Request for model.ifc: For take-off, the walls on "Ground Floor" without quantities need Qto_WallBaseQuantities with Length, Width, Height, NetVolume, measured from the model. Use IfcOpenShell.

First a look at what the model holds.

```python
import ifcopenshell
import ifcopenshell.util.element
import ifcopenshell.util.unit

model = ifcopenshell.open("model.ifc")
print(model.schema)
for unit_type in ("LENGTHUNIT", "AREAUNIT", "VOLUMEUNIT"):
    print(unit_type, ifcopenshell.util.unit.calculate_unit_scale(model, unit_type))
storey = next(s for s in model.by_type("IfcBuildingStorey") if s.Name == "Ground Floor")
walls = [e for e in ifcopenshell.util.element.get_decomposition(storey) if e.is_a("IfcWall")]
for e in sorted(walls, key=lambda e: e.id()):
    print(e.id(), e.is_a(), e.Name, list(ifcopenshell.util.element.get_psets(e, qtos_only=True)), sep=" | ")
```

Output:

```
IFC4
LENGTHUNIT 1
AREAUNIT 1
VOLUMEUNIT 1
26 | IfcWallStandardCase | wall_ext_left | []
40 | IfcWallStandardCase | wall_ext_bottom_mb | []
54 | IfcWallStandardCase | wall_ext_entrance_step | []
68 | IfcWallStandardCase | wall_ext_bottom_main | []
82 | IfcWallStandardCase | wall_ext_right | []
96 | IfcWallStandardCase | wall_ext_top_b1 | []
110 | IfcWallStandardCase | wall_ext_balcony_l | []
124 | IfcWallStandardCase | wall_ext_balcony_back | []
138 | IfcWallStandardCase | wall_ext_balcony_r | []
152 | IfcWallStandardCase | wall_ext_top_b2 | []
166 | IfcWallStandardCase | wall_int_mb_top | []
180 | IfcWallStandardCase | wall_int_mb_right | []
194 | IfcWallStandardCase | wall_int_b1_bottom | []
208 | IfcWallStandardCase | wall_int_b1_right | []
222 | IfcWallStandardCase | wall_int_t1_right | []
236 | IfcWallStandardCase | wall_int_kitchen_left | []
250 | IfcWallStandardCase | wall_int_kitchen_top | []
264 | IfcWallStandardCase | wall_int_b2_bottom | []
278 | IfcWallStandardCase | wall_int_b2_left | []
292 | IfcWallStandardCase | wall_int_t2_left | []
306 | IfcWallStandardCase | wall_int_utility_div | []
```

```python
import ifcopenshell
import ifcopenshell.api.pset
import ifcopenshell.geom
import ifcopenshell.util.element
import ifcopenshell.util.shape
import ifcopenshell.util.unit

model = ifcopenshell.open("model.ifc")
unit_scale = ifcopenshell.util.unit.calculate_unit_scale(model)
volume_scale = ifcopenshell.util.unit.calculate_unit_scale(model, "VOLUMEUNIT")
settings = ifcopenshell.geom.settings()

storey = next(s for s in model.by_type("IfcBuildingStorey") if s.Name == "Ground Floor")
walls = [e for e in ifcopenshell.util.element.get_decomposition(storey) if e.is_a("IfcWall")]

for e in sorted(walls, key=lambda e: e.id()):
    if ifcopenshell.util.element.get_psets(e, qtos_only=True, should_inherit=False):
        continue
    # Geometry comes back in metres, in the element's own axes.
    shape = ifcopenshell.geom.create_shape(settings, e)
    values = {
        "Length": ifcopenshell.util.shape.get_x(shape.geometry) / unit_scale,
        "Width": ifcopenshell.util.shape.get_y(shape.geometry) / unit_scale,
        "Height": ifcopenshell.util.shape.get_z(shape.geometry) / unit_scale,
        "NetVolume": ifcopenshell.util.shape.get_volume(shape.geometry) / volume_scale,
    }
    qto = ifcopenshell.api.pset.add_qto(model, product=e, name="Qto_WallBaseQuantities")
    ifcopenshell.api.pset.edit_qto(model, qto=qto, properties=values)
    print(e.id(), {k: round(v, 3) for k, v in values.items()})

model.write("model_updated.ifc")
```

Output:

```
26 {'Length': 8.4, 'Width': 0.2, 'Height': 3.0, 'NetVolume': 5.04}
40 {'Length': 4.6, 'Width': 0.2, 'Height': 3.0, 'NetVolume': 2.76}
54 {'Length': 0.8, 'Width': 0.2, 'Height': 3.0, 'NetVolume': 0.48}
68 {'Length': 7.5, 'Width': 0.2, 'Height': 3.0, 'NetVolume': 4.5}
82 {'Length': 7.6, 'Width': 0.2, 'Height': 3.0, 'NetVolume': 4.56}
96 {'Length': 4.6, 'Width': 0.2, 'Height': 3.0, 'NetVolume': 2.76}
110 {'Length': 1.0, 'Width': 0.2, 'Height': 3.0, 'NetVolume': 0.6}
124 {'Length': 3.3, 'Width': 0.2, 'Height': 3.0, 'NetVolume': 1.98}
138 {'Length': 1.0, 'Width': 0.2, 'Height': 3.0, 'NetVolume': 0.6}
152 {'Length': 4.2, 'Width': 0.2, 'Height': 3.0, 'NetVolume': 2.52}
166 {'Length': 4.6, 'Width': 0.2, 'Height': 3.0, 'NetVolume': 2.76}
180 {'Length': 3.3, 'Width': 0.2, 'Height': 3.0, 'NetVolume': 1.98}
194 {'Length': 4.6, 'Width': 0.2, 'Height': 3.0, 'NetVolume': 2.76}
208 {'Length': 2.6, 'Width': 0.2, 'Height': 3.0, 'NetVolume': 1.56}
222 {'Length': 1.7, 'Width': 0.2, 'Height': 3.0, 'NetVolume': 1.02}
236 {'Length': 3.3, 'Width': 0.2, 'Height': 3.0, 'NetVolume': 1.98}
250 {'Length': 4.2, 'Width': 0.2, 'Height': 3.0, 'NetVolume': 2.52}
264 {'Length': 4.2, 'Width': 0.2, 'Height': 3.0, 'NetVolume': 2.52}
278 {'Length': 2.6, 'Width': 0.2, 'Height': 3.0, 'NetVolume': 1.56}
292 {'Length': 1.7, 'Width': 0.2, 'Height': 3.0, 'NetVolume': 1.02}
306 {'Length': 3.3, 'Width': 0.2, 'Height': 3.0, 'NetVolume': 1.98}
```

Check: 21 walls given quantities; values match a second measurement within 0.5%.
